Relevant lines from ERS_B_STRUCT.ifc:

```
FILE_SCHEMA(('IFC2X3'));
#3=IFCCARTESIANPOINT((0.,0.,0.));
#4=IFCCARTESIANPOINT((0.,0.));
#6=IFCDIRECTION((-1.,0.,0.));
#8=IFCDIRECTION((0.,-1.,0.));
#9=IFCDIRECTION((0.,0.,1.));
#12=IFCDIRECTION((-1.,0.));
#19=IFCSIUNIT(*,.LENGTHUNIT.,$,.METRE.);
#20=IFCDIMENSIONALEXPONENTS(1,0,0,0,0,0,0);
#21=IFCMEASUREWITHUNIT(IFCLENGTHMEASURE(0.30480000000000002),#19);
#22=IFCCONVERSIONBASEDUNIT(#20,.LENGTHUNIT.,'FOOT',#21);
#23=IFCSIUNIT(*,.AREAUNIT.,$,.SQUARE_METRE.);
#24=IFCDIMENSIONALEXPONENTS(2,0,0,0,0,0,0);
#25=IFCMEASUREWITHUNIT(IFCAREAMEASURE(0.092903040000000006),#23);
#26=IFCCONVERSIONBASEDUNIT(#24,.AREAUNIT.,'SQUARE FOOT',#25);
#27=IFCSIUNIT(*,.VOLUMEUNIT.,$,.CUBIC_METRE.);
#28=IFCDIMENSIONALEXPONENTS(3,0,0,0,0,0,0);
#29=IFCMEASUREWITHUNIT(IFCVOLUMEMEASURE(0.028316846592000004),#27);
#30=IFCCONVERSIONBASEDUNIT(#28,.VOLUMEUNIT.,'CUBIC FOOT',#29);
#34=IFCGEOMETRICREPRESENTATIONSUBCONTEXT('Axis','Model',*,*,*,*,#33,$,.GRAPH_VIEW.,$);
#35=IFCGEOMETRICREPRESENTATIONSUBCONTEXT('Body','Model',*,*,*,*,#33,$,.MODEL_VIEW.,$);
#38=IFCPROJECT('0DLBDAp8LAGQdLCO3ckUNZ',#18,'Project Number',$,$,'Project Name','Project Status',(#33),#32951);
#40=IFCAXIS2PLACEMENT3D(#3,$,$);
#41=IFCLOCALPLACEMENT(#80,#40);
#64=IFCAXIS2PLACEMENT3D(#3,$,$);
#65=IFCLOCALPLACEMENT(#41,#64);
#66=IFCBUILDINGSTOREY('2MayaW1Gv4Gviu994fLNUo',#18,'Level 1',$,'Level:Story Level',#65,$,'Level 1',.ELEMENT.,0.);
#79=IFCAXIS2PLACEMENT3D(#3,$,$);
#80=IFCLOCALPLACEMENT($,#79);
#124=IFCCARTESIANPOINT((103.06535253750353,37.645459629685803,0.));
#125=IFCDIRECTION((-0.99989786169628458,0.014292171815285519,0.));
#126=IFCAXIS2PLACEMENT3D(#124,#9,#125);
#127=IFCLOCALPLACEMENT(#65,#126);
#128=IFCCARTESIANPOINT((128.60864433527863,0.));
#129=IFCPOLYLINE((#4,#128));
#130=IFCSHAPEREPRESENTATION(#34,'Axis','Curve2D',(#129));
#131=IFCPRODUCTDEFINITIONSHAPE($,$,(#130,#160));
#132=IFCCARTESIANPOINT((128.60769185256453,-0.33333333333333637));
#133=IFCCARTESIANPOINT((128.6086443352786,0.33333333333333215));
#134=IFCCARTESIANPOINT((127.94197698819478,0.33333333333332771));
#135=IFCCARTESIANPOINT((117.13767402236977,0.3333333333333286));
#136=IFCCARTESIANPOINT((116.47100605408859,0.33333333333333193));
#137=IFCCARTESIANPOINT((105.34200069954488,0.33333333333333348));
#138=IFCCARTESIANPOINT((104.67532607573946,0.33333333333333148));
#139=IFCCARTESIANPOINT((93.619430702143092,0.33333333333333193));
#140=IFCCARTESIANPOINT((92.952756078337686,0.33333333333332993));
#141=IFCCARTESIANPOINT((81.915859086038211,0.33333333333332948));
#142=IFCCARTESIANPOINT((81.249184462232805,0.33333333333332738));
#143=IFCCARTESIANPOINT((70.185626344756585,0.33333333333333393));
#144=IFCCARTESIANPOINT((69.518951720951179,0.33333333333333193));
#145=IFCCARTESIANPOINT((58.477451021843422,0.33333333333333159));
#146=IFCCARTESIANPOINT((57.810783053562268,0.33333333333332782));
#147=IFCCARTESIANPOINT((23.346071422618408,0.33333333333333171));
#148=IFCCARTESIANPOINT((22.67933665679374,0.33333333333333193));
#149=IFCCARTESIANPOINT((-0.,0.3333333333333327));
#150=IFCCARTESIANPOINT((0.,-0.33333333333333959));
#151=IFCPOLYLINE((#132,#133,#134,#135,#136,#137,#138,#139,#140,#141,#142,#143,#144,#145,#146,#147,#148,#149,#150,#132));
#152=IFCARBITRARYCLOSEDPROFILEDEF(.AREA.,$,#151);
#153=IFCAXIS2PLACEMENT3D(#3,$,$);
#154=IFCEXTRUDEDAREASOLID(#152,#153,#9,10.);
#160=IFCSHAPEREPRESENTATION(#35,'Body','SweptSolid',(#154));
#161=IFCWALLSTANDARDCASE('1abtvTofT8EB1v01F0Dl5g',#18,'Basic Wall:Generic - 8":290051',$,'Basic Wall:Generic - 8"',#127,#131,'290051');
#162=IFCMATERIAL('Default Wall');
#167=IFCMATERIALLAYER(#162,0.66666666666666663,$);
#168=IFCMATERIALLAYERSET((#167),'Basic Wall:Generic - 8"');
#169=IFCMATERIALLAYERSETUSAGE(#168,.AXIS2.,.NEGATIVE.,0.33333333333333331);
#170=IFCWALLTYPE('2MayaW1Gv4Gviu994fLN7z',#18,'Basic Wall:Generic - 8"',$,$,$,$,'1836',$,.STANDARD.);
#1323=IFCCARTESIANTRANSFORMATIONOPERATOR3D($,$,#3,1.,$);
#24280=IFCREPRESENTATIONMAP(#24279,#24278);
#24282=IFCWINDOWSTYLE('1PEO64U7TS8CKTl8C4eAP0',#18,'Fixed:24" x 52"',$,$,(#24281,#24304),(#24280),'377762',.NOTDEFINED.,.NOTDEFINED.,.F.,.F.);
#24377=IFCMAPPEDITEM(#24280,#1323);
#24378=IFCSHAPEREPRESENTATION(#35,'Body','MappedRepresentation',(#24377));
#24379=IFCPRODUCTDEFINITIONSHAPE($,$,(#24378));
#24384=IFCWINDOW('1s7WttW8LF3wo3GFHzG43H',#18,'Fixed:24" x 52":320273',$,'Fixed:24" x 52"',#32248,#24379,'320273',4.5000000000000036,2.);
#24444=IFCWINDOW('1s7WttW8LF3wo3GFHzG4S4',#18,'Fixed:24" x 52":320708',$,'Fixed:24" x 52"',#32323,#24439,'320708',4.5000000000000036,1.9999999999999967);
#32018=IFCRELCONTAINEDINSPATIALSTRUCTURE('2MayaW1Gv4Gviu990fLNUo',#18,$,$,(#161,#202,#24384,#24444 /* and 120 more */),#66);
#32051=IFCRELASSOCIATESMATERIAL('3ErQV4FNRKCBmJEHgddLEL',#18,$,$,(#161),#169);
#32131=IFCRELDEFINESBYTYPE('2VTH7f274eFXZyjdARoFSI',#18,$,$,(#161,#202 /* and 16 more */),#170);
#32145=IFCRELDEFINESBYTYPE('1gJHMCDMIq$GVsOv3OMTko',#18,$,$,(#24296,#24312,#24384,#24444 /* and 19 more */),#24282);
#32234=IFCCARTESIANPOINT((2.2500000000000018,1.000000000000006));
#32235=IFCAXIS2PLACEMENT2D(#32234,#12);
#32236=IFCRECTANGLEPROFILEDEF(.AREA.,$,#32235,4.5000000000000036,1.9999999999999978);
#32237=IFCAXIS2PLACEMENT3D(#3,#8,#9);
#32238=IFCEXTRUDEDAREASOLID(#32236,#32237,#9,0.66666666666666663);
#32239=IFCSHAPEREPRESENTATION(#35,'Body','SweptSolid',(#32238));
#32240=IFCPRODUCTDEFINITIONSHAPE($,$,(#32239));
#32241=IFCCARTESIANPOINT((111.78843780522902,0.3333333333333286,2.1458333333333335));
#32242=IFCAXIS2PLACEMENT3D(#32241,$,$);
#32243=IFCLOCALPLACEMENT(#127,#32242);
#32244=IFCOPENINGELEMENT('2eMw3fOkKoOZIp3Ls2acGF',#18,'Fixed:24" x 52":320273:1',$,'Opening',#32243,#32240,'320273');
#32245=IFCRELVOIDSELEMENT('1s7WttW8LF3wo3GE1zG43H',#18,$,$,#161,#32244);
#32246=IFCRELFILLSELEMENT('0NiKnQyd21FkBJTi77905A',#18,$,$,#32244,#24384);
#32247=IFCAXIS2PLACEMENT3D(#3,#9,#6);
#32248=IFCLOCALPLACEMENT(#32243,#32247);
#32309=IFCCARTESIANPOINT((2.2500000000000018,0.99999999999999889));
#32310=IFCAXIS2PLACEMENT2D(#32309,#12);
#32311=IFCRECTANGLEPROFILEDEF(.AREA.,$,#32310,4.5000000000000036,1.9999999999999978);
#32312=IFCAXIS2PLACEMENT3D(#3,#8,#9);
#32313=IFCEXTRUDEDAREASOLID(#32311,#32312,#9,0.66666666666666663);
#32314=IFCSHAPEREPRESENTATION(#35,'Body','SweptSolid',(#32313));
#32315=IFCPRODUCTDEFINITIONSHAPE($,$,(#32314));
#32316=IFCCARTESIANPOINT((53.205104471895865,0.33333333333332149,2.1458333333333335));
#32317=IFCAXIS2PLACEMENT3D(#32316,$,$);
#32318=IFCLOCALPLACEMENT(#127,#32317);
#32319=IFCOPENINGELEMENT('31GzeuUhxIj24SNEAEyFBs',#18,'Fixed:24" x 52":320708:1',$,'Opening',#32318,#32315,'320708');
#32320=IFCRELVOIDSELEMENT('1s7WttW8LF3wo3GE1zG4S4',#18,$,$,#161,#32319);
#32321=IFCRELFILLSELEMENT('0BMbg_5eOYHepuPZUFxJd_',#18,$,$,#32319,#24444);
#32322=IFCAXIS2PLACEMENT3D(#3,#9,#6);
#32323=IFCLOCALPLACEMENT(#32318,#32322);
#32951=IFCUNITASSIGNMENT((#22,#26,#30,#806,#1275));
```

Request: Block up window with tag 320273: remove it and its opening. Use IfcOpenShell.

```python
import ifcopenshell
import ifcopenshell.api.feature
import ifcopenshell.api.root
import ifcopenshell.geom
import ifcopenshell.util.shape

model = ifcopenshell.open("ERS_B_STRUCT.ifc")
settings = ifcopenshell.geom.settings()


def volume(element):
    """Net volume in cubic metres, openings subtracted."""
    shape = ifcopenshell.geom.create_shape(settings, element)
    return ifcopenshell.util.shape.get_volume(shape.geometry)


window = model.by_id(24384)
opening = window.FillsVoids[0].RelatingOpeningElement
wall = opening.VoidsElements[0].RelatingBuildingElement
before = volume(wall)

ifcopenshell.api.root.remove_product(model, product=window)
ifcopenshell.api.feature.remove_feature(model, feature=opening)

after = volume(wall)

print(f"wall volume {before:.3f} -> {after:.3f} m3")

model.write("ERS_B_STRUCT_updated.ifc")
```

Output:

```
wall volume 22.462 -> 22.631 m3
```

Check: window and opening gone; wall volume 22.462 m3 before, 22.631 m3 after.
